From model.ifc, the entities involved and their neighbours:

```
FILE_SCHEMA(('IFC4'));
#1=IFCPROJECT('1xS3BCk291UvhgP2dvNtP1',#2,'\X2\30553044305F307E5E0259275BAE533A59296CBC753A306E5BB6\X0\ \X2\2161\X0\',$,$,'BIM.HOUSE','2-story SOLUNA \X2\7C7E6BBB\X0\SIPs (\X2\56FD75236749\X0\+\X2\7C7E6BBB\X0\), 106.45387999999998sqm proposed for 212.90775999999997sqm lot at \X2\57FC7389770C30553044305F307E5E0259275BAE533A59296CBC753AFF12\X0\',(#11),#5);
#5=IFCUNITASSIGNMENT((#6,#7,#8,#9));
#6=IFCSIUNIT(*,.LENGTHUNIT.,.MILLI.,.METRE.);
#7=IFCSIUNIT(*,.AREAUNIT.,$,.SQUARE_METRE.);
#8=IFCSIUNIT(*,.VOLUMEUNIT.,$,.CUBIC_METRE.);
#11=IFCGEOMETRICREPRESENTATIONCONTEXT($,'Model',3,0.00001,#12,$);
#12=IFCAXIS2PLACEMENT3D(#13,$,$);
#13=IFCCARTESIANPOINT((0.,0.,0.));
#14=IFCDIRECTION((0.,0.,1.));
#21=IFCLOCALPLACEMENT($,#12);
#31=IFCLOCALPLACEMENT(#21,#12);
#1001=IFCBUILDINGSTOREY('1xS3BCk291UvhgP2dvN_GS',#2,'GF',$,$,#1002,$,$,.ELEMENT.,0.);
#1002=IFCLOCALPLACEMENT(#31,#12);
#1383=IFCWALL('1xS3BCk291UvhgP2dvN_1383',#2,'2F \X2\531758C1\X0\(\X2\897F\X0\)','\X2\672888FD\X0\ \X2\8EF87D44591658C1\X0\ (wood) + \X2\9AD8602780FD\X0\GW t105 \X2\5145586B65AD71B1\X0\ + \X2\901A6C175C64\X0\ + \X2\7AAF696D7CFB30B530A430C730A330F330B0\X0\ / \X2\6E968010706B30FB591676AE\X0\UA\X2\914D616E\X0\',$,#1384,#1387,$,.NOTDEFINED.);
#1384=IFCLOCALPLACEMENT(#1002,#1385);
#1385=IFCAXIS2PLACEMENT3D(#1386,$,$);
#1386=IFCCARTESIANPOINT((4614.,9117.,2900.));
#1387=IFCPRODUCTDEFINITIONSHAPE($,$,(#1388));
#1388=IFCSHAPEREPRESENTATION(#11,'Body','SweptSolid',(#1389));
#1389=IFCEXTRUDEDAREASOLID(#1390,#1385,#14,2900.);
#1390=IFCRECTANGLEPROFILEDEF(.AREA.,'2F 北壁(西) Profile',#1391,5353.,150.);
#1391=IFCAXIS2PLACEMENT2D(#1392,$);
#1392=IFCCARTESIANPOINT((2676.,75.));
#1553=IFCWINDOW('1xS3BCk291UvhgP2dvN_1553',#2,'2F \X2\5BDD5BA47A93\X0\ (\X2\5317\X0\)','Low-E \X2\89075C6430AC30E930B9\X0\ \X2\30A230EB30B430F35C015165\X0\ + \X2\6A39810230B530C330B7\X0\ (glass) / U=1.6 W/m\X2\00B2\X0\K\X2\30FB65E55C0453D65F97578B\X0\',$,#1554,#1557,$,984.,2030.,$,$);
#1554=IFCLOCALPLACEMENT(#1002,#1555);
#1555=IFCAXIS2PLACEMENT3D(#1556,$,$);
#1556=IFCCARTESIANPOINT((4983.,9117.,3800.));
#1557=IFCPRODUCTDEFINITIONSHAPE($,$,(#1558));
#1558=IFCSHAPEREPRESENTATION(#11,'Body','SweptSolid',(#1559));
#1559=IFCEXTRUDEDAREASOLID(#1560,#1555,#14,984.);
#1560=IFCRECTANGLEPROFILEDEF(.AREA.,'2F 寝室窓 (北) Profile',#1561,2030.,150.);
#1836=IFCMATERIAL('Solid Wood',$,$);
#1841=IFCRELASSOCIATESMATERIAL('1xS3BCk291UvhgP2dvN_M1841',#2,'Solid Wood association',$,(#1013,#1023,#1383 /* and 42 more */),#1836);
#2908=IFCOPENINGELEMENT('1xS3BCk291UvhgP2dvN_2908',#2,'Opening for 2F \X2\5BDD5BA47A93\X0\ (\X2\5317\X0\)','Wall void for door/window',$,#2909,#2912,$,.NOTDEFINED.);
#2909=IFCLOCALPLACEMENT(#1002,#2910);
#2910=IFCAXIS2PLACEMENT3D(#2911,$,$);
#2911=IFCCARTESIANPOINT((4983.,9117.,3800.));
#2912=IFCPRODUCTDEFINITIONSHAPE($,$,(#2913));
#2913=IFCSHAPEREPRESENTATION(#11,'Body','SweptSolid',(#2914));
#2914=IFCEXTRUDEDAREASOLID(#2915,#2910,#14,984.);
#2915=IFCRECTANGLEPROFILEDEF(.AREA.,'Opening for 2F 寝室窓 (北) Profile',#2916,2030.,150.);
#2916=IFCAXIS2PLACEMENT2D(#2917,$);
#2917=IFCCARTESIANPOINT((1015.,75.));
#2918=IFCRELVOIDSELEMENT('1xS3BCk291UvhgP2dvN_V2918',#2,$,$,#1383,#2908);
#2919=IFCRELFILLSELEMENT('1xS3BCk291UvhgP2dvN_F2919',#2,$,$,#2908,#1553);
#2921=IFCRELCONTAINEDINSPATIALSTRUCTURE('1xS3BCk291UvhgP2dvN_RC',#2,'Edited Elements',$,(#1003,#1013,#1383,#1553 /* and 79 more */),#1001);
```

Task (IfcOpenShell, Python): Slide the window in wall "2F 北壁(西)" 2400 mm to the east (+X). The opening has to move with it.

```python
import ifcopenshell
import ifcopenshell.api.geometry
import ifcopenshell.util.placement
import ifcopenshell.util.unit

model = ifcopenshell.open("model.ifc")
unit_scale = ifcopenshell.util.unit.calculate_unit_scale(model)

window = model.by_guid("1xS3BCk291UvhgP2dvN_1553")
opening = window.FillsVoids[0].RelatingOpeningElement
wall = opening.VoidsElements[0].RelatingBuildingElement

wall_matrix = ifcopenshell.util.placement.get_local_placement(wall.ObjectPlacement)
shift = wall_matrix[:3, 0] * 2.4 / unit_scale
before = ifcopenshell.util.placement.get_local_placement(window.ObjectPlacement)[:3, 3].copy()

# The window is not placed relative to its opening, so move both.
for product in (opening, window):
    matrix = ifcopenshell.util.placement.get_local_placement(product.ObjectPlacement)
    matrix[:3, 3] += shift
    ifcopenshell.api.geometry.edit_object_placement(model, product=product, matrix=matrix, is_si=False)

after = ifcopenshell.util.placement.get_local_placement(window.ObjectPlacement)[:3, 3]
print("window moved by", (after - before).round(3) + 0.0)

model.write("model_rev.ifc")
```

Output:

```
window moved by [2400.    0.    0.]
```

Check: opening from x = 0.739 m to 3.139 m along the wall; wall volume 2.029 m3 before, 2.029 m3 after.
